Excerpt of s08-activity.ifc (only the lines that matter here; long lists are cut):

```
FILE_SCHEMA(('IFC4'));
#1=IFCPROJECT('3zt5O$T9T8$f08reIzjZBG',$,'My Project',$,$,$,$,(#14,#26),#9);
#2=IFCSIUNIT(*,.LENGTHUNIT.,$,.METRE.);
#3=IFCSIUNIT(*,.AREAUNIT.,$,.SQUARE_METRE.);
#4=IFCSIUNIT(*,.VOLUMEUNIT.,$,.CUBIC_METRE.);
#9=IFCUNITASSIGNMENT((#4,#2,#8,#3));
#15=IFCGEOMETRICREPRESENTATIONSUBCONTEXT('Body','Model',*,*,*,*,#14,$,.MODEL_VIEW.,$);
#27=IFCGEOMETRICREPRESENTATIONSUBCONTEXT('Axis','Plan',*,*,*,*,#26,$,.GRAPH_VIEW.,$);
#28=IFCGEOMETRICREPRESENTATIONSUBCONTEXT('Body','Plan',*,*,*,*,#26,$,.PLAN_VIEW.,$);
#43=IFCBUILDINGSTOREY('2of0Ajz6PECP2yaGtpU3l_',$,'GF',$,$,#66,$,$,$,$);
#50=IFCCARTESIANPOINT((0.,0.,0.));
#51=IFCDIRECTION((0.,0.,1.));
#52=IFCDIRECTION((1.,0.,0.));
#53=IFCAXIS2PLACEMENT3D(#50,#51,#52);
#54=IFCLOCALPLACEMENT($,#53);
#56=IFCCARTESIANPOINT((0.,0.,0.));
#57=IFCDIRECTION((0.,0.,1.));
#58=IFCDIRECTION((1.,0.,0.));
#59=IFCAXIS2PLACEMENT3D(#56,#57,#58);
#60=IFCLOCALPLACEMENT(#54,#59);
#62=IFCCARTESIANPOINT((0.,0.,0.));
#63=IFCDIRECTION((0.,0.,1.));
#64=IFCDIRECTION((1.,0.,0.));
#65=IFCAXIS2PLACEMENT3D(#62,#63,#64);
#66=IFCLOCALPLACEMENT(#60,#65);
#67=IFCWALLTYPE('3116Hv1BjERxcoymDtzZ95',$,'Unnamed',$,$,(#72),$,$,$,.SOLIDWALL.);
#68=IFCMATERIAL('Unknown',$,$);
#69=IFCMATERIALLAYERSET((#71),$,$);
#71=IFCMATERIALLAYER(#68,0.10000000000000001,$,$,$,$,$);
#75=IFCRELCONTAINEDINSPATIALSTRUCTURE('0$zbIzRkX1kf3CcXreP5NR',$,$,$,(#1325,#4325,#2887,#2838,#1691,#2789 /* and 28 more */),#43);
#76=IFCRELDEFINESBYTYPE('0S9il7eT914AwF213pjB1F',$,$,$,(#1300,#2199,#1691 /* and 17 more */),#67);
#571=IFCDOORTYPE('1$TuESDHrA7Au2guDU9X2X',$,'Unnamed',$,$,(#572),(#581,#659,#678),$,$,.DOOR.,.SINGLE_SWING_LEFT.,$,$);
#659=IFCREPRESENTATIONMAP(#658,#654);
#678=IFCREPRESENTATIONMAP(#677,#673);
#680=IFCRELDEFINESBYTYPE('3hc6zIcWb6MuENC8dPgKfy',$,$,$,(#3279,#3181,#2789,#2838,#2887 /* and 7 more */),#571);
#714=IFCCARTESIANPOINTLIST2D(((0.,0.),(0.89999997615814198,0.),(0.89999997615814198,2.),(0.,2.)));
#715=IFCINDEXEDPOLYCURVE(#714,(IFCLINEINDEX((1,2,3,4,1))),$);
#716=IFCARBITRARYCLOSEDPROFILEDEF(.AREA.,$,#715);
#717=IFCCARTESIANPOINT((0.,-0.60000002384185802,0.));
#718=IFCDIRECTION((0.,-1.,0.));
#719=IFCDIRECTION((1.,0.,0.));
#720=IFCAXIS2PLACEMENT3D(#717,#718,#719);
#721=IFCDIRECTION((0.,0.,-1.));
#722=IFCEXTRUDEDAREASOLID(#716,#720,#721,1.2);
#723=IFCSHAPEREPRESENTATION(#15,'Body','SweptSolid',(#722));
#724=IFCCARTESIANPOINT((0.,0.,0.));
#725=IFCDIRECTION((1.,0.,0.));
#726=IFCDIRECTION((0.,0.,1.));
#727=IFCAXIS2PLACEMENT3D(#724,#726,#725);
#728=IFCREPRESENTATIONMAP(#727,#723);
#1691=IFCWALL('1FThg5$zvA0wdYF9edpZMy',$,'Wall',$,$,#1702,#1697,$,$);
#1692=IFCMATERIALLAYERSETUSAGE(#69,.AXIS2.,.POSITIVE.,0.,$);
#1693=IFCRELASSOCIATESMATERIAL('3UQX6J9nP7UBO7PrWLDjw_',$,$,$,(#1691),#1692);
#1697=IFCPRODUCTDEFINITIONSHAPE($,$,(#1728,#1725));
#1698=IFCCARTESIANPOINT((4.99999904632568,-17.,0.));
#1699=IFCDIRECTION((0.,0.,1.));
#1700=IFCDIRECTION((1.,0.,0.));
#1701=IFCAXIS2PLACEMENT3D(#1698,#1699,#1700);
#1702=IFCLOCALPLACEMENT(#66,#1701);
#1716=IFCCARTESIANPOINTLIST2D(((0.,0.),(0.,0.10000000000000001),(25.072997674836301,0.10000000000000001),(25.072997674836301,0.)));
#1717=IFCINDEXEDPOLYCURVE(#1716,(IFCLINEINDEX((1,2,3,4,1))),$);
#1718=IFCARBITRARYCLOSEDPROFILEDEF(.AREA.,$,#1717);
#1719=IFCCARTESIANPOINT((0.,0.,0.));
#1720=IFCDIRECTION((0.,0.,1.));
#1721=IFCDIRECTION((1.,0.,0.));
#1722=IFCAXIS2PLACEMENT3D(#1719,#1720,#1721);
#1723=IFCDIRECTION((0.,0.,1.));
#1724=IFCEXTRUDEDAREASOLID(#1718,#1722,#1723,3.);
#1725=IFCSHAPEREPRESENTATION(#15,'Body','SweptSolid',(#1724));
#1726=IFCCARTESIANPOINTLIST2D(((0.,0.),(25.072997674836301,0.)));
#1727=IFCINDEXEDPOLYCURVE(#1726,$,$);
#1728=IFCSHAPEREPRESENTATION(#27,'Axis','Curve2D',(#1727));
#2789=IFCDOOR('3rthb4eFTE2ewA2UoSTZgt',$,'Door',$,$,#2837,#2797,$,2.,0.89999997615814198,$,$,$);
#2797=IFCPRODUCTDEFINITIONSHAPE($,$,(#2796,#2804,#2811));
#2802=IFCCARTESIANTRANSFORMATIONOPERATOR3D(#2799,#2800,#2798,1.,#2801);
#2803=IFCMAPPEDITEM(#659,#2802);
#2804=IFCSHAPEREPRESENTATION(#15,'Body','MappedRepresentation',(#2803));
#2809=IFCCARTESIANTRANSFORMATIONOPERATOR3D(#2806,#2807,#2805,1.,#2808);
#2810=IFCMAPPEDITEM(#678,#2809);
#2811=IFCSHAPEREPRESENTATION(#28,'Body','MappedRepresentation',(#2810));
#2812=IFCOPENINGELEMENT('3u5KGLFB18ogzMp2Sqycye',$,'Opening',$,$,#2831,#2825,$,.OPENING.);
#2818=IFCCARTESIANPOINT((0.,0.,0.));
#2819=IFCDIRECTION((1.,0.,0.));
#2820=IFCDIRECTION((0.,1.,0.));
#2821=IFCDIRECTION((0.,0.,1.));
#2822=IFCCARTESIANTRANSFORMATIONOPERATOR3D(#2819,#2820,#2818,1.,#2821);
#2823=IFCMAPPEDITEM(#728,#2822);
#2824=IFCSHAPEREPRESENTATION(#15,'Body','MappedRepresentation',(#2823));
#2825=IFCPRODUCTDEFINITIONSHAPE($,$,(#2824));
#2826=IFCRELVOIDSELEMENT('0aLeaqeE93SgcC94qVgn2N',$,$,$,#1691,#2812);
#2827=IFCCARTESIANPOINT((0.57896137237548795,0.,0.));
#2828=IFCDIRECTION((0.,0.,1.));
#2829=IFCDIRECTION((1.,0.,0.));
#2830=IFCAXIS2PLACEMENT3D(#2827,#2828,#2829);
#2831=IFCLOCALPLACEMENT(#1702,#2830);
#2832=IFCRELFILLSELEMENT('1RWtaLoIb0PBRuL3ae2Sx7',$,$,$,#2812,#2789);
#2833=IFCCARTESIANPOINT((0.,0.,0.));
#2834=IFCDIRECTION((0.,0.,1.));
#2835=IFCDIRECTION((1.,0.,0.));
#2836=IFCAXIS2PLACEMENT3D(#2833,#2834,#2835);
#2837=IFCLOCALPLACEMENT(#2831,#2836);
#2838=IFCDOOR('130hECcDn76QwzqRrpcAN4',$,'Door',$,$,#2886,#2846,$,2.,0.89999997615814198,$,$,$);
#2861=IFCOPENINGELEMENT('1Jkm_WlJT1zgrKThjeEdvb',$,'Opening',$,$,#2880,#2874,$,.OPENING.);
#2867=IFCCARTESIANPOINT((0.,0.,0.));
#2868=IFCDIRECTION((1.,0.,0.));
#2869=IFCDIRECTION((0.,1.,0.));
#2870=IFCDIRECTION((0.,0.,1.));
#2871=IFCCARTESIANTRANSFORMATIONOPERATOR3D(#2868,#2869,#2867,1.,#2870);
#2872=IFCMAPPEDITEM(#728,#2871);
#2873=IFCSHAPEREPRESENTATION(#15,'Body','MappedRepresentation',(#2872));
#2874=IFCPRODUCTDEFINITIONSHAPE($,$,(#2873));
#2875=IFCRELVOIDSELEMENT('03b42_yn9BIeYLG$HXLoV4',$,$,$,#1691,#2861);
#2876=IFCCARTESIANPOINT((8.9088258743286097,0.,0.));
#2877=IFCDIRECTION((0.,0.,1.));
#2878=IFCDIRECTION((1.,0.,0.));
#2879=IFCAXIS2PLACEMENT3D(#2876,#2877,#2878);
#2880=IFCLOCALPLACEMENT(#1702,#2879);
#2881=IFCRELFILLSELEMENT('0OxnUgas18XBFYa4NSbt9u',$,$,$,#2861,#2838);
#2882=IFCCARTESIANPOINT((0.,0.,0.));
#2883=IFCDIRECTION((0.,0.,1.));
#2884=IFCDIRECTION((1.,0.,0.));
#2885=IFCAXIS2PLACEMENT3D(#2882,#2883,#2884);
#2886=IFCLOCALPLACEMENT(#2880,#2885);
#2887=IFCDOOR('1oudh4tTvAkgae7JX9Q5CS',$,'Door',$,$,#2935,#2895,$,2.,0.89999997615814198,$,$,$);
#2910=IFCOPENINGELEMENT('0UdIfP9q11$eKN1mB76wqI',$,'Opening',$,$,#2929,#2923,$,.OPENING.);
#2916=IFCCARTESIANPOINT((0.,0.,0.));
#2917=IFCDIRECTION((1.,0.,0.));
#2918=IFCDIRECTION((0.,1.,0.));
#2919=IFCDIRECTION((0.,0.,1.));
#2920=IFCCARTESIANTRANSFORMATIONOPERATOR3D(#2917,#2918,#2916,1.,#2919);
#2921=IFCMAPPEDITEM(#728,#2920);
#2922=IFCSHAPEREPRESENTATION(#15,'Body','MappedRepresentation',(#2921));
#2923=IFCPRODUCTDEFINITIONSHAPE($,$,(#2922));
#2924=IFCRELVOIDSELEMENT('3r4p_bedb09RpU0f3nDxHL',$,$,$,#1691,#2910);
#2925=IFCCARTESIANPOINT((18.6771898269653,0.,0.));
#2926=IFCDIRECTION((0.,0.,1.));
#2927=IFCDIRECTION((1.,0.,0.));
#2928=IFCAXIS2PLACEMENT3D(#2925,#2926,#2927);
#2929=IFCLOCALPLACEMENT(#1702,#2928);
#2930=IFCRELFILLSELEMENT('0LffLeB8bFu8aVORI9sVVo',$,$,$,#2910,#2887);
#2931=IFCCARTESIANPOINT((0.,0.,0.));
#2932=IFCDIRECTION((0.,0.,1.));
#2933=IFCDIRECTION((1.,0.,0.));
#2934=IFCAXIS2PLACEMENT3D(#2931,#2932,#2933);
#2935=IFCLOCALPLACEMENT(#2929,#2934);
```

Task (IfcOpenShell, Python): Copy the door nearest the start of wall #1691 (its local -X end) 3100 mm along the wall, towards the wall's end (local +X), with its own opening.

```python
import ifcopenshell
import ifcopenshell.api.feature
import ifcopenshell.api.geometry
import ifcopenshell.api.root
import ifcopenshell.geom
import ifcopenshell.util.element
import ifcopenshell.util.placement
import ifcopenshell.util.shape
import ifcopenshell.util.unit

model = ifcopenshell.open("s08-activity.ifc")
unit_scale = ifcopenshell.util.unit.calculate_unit_scale(model)
settings = ifcopenshell.geom.settings()


def volume(element):
    """Net volume in cubic metres, openings subtracted."""
    shape = ifcopenshell.geom.create_shape(settings, element)
    return ifcopenshell.util.shape.get_volume(shape.geometry)


door = model.by_id(2789)
opening = door.FillsVoids[0].RelatingOpeningElement
wall = opening.VoidsElements[0].RelatingBuildingElement
before = volume(wall)
shift = ifcopenshell.util.placement.get_local_placement(wall.ObjectPlacement)[:3, 0] * 3.1 / unit_scale

# copy_class copies the void relationship, type, container and properties, but no geometry.
new_opening = ifcopenshell.api.root.copy_class(model, product=opening)
new_opening.Representation = ifcopenshell.util.element.copy_deep(
    model, opening.Representation, exclude=["IfcGeometricRepresentationContext", "IfcRepresentationMap"]
)
new_door = ifcopenshell.api.root.copy_class(model, product=door)
new_door.Representation = ifcopenshell.util.element.copy_deep(
    model, door.Representation, exclude=["IfcGeometricRepresentationContext", "IfcRepresentationMap"]
)
ifcopenshell.api.feature.add_filling(model, opening=new_opening, element=new_door)

for old, new in ((opening, new_opening), (door, new_door)):
    matrix = ifcopenshell.util.placement.get_local_placement(old.ObjectPlacement)
    matrix[:3, 3] += shift
    ifcopenshell.api.geometry.edit_object_placement(model, product=new, matrix=matrix, is_si=False)

after = volume(wall)

print(f"wall volume {before:.3f} -> {after:.3f} m3")

model.write("s08-activity_edited.ifc")
```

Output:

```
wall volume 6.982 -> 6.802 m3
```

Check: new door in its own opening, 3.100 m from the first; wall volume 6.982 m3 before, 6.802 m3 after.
